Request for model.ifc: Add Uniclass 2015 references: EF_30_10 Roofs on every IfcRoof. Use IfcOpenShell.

First a look at what the model holds.

```python
import ifcopenshell

model = ifcopenshell.open("model.ifc")
print(model.schema)
print("classifications:", [c.Name for c in model.by_type("IfcClassification")])
for ifc_class in ("IfcDoor", "IfcRoof", "IfcStair", "IfcWall", "IfcWindow"):
    print(ifc_class, len(model.by_type(ifc_class)))
```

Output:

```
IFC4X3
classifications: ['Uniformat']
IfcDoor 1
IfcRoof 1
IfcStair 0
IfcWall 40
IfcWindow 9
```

```python
import ifcopenshell
import ifcopenshell.api.classification

model = ifcopenshell.open("model.ifc")

system = ifcopenshell.api.classification.add_classification(model, classification="Uniclass 2015")

codes = {
    "IfcRoof": ("EF_30_10", "Roofs"),
}
for ifc_class, (code, name) in codes.items():
    products = model.by_type(ifc_class)
    ifcopenshell.api.classification.add_reference(
        model, products=products, classification=system, identification=code, name=name
    )
    print(code, len(products))

model.write("model_v2.ifc")
```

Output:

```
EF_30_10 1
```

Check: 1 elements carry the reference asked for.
